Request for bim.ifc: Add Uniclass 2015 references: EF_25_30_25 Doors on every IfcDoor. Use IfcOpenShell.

First a look at what the model holds.

```python
import ifcopenshell

model = ifcopenshell.open("bim.ifc")
print(model.schema)
print("classifications:", [c.Name for c in model.by_type("IfcClassification")])
for ifc_class in ("IfcDoor", "IfcRoof", "IfcStair", "IfcWall", "IfcWindow"):
    print(ifc_class, len(model.by_type(ifc_class)))
```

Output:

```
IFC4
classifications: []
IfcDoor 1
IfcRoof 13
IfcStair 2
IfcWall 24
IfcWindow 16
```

```python
import ifcopenshell
import ifcopenshell.api.classification

model = ifcopenshell.open("bim.ifc")

system = ifcopenshell.api.classification.add_classification(model, classification="Uniclass 2015")

codes = {
    "IfcDoor": ("EF_25_30_25", "Doors"),
}
for ifc_class, (code, name) in codes.items():
    products = model.by_type(ifc_class)
    ifcopenshell.api.classification.add_reference(
        model, products=products, classification=system, identification=code, name=name
    )
    print(code, len(products))

model.write("bim_edited.ifc")
```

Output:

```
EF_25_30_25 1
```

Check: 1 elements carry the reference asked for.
